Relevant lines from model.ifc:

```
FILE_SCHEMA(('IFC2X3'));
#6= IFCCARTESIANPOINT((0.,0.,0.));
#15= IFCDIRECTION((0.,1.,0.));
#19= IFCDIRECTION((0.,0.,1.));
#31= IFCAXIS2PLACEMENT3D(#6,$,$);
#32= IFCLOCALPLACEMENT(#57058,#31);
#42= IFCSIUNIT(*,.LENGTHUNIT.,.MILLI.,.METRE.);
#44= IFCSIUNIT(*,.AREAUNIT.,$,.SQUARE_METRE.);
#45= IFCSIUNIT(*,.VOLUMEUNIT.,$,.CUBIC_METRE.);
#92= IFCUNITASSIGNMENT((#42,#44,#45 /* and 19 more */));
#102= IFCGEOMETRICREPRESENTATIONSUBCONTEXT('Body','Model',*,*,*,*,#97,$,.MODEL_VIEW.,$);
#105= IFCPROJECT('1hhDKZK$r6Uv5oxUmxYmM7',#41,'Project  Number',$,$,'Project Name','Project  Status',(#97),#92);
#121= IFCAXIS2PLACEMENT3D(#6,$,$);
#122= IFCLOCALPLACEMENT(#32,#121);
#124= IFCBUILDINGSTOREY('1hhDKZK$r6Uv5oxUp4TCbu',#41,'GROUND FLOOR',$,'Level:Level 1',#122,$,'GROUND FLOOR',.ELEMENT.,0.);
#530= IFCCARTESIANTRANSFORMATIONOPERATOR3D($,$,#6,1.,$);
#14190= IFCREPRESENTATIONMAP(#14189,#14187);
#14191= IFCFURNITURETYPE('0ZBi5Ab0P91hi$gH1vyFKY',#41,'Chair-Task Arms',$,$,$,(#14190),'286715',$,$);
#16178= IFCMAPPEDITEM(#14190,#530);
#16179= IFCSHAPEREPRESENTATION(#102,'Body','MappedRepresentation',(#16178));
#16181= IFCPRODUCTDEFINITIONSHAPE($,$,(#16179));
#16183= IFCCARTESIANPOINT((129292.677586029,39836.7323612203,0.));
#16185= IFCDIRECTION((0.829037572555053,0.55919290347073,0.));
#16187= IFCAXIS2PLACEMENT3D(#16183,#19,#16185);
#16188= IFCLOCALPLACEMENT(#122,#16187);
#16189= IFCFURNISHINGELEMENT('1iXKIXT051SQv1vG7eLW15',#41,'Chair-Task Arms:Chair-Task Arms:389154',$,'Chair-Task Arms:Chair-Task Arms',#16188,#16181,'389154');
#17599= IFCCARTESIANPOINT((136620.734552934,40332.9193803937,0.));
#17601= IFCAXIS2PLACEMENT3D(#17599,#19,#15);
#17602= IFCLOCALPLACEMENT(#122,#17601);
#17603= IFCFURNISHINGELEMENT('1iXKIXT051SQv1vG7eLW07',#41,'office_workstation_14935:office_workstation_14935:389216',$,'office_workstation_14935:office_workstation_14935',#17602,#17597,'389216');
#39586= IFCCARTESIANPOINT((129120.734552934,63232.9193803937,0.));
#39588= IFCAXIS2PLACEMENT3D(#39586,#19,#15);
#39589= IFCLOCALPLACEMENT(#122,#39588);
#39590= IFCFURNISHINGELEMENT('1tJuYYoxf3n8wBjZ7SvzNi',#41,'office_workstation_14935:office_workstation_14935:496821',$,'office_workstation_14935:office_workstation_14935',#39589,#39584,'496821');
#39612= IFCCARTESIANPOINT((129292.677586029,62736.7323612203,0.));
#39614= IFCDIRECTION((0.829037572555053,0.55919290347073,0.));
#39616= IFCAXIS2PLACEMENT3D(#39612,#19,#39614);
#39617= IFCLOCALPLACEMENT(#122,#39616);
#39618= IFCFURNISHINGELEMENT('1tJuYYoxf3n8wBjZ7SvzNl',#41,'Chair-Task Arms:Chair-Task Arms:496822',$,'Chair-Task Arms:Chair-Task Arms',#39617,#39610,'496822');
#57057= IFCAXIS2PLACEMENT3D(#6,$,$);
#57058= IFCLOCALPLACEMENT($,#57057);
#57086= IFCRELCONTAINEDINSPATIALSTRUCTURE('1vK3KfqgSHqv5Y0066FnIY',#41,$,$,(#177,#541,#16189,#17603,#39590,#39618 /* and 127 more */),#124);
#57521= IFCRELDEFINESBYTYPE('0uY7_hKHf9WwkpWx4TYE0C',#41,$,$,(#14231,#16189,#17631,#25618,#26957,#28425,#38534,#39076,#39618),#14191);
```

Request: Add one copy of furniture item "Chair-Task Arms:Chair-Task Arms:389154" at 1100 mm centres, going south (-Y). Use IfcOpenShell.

```python
import numpy as np
import ifcopenshell
import ifcopenshell.api.geometry
import ifcopenshell.api.root
import ifcopenshell.util.element
import ifcopenshell.util.placement

model = ifcopenshell.open("model.ifc")


def reuse_history(source, copy):
    """copy_class also copies each property set's owner history, people and application; keep the originals."""
    for rel in copy.IsDefinedBy:
        if rel.is_a("IfcRelDefinesByProperties") and (history := rel.RelatingPropertyDefinition.OwnerHistory):
            rel.RelatingPropertyDefinition.OwnerHistory = source.OwnerHistory
            ifcopenshell.util.element.remove_deep2(model, history)


source = model.by_guid("1iXKIXT051SQv1vG7eLW15")
base = ifcopenshell.util.placement.get_local_placement(source.ObjectPlacement)
step = np.array([0.0, -1.0, 0.0]) * 1100.0

for i in range(1, 2):
    copy = ifcopenshell.api.root.copy_class(model, product=source)
    copy.Representation = ifcopenshell.util.element.copy_deep(
        model, source.Representation, exclude=["IfcGeometricRepresentationContext", "IfcRepresentationMap"]
    )
    copy.Name = "Chair-Task Arms:Chair-Task Arms"
    copy.Tag = None
    reuse_history(source, copy)
    matrix = base.copy()
    matrix[:3, 3] += i * step
    print("added at", matrix[:3, 3].round(3) + 0.0)
    ifcopenshell.api.geometry.edit_object_placement(model, product=copy, matrix=matrix, is_si=False)

model.write("model-out.ifc")
```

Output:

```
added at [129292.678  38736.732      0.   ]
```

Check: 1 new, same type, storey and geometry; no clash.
